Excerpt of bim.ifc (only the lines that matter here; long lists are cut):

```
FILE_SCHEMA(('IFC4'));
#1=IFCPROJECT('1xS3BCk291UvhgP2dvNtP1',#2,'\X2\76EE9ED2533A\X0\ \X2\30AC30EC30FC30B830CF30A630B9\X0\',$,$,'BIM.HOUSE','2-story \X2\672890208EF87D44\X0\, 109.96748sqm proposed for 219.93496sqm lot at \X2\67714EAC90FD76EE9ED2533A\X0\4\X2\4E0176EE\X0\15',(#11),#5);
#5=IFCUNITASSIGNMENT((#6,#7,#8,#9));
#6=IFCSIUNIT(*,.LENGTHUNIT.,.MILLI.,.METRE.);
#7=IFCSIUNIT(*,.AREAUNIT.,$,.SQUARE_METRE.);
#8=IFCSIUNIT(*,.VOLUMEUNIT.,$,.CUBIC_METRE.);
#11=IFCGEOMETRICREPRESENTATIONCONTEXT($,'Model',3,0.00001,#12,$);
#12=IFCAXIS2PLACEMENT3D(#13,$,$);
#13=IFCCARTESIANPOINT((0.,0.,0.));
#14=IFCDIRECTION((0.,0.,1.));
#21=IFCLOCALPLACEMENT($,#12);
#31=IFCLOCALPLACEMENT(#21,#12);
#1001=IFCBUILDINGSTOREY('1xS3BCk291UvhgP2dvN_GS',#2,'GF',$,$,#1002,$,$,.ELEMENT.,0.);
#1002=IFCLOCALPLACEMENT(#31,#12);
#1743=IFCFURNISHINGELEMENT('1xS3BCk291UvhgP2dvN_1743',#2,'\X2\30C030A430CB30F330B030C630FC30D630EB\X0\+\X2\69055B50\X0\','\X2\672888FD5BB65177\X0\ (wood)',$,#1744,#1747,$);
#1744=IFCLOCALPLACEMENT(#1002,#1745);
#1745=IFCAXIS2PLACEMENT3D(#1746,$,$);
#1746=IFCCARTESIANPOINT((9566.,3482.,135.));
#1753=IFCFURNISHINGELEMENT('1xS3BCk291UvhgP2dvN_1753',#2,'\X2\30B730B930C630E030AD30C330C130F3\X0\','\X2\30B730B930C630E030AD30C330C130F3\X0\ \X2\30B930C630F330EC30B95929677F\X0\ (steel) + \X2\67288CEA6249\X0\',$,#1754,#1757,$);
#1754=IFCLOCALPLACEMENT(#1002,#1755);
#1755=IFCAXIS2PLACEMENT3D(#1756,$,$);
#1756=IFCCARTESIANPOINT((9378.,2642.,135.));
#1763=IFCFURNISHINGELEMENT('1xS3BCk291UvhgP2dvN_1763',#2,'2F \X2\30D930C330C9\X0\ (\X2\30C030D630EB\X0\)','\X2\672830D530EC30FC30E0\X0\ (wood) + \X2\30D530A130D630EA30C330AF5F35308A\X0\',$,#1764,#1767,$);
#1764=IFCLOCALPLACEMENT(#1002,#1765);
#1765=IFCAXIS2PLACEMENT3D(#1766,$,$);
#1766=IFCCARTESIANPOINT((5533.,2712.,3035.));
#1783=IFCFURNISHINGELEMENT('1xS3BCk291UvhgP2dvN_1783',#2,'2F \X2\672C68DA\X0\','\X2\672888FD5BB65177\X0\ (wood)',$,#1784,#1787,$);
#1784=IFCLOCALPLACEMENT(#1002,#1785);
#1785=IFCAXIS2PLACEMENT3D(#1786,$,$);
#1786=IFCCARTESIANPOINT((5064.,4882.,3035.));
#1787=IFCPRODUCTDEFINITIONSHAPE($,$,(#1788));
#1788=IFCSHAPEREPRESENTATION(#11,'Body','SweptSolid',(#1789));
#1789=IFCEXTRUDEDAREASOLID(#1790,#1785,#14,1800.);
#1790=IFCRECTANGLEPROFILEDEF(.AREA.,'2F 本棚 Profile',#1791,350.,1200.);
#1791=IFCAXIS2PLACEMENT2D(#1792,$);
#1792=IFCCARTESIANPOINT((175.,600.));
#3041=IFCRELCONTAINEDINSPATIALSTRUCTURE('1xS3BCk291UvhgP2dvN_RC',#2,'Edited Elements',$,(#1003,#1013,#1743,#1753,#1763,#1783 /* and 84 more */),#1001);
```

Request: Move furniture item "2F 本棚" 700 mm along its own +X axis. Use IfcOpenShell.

```python
import ifcopenshell
import ifcopenshell.api.geometry
import ifcopenshell.util.placement
import ifcopenshell.util.unit

model = ifcopenshell.open("bim.ifc")
unit_scale = ifcopenshell.util.unit.calculate_unit_scale(model)

item = model.by_guid("1xS3BCk291UvhgP2dvN_1783")
matrix = ifcopenshell.util.placement.get_local_placement(item.ObjectPlacement)
matrix[:3, 3] += matrix[:3, 0] * 0.7 / unit_scale
ifcopenshell.api.geometry.edit_object_placement(model, product=item, matrix=matrix, is_si=False)

print(ifcopenshell.util.placement.get_local_placement(item.ObjectPlacement).round(3) + 0.0)

model.write("bim-out.ifc")
```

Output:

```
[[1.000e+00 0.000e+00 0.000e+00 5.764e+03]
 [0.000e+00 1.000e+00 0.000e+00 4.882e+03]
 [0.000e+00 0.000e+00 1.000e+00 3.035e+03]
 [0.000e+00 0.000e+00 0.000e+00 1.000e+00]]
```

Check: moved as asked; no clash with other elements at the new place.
